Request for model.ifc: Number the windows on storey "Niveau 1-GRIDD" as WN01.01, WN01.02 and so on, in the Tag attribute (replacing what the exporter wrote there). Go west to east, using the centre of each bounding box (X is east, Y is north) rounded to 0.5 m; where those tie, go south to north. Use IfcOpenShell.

First a look at what the model holds.

```python
import ifcopenshell
import ifcopenshell.util.element
import ifcopenshell.util.placement

model = ifcopenshell.open("model.ifc")
print(model.schema)
storey = next(s for s in model.by_type("IfcBuildingStorey") if s.Name == "Niveau 1-GRIDD")
windows = [e for e in ifcopenshell.util.element.get_decomposition(storey) if e.is_a("IfcWindow")]
for e in sorted(windows, key=lambda e: e.id()):
    origin = ifcopenshell.util.placement.get_local_placement(e.ObjectPlacement)[:3, 3]
    print(e.id(), e.Tag, e.Name, origin.round(2) + 0.0, sep=" | ")
```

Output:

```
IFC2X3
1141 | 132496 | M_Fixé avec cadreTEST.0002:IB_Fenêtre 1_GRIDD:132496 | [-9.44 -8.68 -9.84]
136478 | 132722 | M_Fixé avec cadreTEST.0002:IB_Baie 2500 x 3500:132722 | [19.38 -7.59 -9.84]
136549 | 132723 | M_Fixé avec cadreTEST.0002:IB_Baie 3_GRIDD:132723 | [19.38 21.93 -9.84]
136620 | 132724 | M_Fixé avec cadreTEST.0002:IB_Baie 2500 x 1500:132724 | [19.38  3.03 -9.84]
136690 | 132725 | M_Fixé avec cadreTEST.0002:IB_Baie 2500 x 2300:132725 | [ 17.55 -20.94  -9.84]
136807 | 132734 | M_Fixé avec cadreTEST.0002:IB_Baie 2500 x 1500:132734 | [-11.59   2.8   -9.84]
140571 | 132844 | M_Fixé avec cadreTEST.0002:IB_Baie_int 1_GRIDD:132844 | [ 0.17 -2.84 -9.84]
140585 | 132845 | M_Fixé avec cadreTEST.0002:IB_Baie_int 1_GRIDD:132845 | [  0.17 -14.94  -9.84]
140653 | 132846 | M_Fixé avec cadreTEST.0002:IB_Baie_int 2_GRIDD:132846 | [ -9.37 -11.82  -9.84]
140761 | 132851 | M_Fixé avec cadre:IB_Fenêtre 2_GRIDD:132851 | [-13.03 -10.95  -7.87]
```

```python
import ifcopenshell
import ifcopenshell.geom
import ifcopenshell.util.element
import ifcopenshell.util.shape

model = ifcopenshell.open("model.ifc")
settings = ifcopenshell.geom.settings()
settings.set("use-world-coords", True)


def centre(element):
    shape = ifcopenshell.geom.create_shape(settings, element)
    return ifcopenshell.util.shape.get_bbox_centroid(shape.geometry)


storey = next(s for s in model.by_type("IfcBuildingStorey") if s.Name == "Niveau 1-GRIDD")
windows = [e for e in ifcopenshell.util.element.get_decomposition(storey) if e.is_a("IfcWindow")]

# Insertion points can sit at a corner or the storey origin, so sort by the geometry (in metres).
centres = {e: centre(e) for e in windows}
windows.sort(key=lambda e: (round(centres[e][0] / 0.5), centres[e][1]))

for i, e in enumerate(windows, start=1):
    number = f"WN01.{i:02d}"
    e.Tag = number
    print(e.id(), number)

model.write("model_updated.ifc")
```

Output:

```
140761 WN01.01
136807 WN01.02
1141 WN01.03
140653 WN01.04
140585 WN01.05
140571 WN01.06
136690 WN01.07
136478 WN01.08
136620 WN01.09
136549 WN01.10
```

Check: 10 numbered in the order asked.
